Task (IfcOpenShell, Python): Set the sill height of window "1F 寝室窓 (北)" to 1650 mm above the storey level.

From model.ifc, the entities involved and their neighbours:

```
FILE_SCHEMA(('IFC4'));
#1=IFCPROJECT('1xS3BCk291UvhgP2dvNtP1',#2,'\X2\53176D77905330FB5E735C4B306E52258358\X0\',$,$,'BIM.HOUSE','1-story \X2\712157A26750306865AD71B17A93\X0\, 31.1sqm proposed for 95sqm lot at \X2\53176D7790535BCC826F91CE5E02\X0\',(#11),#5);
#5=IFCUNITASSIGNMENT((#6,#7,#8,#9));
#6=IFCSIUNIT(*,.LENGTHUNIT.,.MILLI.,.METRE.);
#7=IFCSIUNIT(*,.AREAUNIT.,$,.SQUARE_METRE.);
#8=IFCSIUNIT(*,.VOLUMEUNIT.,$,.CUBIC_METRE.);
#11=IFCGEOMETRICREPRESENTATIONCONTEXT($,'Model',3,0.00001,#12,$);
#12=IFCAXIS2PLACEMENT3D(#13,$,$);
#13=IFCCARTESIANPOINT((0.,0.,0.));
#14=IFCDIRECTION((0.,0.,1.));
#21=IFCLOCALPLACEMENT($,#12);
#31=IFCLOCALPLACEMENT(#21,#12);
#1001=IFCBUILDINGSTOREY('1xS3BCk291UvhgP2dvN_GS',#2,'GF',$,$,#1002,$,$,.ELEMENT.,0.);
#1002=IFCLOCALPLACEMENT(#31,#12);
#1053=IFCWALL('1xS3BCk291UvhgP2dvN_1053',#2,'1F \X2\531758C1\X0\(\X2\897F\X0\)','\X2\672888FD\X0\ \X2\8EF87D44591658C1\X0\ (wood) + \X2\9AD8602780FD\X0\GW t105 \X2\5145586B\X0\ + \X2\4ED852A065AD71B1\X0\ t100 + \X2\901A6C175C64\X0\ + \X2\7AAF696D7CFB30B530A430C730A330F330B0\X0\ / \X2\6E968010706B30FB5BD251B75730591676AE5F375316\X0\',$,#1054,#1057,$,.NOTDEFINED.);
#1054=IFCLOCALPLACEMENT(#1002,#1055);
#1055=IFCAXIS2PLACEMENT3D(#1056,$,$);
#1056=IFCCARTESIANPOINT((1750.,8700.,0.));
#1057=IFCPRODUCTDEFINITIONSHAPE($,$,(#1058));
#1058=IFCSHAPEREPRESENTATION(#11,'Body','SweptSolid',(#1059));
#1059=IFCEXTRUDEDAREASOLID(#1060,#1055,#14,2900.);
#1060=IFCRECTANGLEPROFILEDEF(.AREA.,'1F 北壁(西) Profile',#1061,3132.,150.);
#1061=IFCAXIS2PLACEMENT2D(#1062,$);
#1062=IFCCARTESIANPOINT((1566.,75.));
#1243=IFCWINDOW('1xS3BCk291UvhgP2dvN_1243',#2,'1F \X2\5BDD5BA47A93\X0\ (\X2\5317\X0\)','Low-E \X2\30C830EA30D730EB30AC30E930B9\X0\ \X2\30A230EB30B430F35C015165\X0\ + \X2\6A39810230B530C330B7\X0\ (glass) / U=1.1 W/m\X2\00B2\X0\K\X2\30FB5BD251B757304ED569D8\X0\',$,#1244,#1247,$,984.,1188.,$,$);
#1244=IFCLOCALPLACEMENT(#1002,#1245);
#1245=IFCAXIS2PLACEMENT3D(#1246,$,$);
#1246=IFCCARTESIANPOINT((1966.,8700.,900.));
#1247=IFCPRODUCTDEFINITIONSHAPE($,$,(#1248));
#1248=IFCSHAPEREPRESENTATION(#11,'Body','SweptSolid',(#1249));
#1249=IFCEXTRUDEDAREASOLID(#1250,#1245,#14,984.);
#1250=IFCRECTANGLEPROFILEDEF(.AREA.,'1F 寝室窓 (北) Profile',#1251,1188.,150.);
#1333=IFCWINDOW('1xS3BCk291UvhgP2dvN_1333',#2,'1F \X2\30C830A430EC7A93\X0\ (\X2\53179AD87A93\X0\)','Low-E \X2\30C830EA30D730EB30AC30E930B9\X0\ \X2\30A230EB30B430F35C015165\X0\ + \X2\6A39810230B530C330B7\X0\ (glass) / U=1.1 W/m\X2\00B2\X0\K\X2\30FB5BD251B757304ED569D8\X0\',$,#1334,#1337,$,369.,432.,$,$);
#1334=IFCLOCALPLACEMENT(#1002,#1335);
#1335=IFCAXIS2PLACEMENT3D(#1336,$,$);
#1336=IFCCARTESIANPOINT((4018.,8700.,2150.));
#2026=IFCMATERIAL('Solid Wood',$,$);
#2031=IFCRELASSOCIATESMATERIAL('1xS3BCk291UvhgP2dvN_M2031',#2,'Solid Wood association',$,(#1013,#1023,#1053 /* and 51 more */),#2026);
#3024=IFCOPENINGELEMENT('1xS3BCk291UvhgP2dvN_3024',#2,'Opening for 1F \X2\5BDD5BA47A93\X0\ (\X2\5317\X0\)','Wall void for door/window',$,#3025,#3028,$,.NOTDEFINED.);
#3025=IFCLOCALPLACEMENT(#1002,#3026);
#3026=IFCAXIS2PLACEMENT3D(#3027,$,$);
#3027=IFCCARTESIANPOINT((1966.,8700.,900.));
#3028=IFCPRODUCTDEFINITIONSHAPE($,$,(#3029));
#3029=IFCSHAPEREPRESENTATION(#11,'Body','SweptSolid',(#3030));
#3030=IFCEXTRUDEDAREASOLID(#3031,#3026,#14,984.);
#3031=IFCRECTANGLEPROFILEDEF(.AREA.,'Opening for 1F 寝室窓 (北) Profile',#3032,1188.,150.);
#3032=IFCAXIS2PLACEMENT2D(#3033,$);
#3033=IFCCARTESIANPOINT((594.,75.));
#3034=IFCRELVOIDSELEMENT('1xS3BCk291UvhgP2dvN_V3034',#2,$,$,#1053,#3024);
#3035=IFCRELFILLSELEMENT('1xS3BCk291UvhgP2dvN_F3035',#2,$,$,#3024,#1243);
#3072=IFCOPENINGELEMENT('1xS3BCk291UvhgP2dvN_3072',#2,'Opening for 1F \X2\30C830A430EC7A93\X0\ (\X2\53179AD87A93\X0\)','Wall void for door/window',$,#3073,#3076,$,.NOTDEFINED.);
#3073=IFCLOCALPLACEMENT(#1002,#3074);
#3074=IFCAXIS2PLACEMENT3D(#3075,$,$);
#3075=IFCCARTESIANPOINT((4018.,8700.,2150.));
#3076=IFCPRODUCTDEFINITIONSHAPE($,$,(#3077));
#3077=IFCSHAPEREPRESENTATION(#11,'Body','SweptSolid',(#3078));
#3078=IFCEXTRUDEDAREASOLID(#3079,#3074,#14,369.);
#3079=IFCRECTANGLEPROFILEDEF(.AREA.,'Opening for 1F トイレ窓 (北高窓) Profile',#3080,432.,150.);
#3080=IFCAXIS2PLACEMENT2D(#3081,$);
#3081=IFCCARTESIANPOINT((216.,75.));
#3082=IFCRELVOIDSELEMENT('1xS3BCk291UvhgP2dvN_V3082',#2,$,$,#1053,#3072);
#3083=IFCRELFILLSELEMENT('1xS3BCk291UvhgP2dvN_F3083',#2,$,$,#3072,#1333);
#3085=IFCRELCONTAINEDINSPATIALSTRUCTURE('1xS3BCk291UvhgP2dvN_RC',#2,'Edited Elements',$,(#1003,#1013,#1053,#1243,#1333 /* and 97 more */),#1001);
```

```python
import numpy as np
import ifcopenshell
import ifcopenshell.api.geometry
import ifcopenshell.geom
import ifcopenshell.util.element
import ifcopenshell.util.placement
import ifcopenshell.util.shape
import ifcopenshell.util.unit

model = ifcopenshell.open("model.ifc")
unit_scale = ifcopenshell.util.unit.calculate_unit_scale(model)

window = model.by_guid("1xS3BCk291UvhgP2dvN_1243")
opening = window.FillsVoids[0].RelatingOpeningElement
storey = ifcopenshell.util.element.get_container(window, ifc_class="IfcBuildingStorey")
level = ifcopenshell.util.placement.get_local_placement(storey.ObjectPlacement)[2, 3]

# The opening's origin need not be at the sill, so measure its lowest point.
shape = ifcopenshell.geom.create_shape(ifcopenshell.geom.settings(), opening)
bottom = ifcopenshell.util.shape.get_shape_bottom_elevation(shape, shape.geometry) / unit_scale
dz = level + 1.65 / unit_scale - bottom

shift = np.array([0.0, 0.0, dz])
# The window is not placed relative to its opening, so move both.
for product in (opening, window):
    matrix = ifcopenshell.util.placement.get_local_placement(product.ObjectPlacement)
    matrix[:3, 3] += shift
    ifcopenshell.api.geometry.edit_object_placement(model, product=product, matrix=matrix, is_si=False)

print(f"moved by {dz * unit_scale:+.3f} m")

model.write("model_updated.ifc")
```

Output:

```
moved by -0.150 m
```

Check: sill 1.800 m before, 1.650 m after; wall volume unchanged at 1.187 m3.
